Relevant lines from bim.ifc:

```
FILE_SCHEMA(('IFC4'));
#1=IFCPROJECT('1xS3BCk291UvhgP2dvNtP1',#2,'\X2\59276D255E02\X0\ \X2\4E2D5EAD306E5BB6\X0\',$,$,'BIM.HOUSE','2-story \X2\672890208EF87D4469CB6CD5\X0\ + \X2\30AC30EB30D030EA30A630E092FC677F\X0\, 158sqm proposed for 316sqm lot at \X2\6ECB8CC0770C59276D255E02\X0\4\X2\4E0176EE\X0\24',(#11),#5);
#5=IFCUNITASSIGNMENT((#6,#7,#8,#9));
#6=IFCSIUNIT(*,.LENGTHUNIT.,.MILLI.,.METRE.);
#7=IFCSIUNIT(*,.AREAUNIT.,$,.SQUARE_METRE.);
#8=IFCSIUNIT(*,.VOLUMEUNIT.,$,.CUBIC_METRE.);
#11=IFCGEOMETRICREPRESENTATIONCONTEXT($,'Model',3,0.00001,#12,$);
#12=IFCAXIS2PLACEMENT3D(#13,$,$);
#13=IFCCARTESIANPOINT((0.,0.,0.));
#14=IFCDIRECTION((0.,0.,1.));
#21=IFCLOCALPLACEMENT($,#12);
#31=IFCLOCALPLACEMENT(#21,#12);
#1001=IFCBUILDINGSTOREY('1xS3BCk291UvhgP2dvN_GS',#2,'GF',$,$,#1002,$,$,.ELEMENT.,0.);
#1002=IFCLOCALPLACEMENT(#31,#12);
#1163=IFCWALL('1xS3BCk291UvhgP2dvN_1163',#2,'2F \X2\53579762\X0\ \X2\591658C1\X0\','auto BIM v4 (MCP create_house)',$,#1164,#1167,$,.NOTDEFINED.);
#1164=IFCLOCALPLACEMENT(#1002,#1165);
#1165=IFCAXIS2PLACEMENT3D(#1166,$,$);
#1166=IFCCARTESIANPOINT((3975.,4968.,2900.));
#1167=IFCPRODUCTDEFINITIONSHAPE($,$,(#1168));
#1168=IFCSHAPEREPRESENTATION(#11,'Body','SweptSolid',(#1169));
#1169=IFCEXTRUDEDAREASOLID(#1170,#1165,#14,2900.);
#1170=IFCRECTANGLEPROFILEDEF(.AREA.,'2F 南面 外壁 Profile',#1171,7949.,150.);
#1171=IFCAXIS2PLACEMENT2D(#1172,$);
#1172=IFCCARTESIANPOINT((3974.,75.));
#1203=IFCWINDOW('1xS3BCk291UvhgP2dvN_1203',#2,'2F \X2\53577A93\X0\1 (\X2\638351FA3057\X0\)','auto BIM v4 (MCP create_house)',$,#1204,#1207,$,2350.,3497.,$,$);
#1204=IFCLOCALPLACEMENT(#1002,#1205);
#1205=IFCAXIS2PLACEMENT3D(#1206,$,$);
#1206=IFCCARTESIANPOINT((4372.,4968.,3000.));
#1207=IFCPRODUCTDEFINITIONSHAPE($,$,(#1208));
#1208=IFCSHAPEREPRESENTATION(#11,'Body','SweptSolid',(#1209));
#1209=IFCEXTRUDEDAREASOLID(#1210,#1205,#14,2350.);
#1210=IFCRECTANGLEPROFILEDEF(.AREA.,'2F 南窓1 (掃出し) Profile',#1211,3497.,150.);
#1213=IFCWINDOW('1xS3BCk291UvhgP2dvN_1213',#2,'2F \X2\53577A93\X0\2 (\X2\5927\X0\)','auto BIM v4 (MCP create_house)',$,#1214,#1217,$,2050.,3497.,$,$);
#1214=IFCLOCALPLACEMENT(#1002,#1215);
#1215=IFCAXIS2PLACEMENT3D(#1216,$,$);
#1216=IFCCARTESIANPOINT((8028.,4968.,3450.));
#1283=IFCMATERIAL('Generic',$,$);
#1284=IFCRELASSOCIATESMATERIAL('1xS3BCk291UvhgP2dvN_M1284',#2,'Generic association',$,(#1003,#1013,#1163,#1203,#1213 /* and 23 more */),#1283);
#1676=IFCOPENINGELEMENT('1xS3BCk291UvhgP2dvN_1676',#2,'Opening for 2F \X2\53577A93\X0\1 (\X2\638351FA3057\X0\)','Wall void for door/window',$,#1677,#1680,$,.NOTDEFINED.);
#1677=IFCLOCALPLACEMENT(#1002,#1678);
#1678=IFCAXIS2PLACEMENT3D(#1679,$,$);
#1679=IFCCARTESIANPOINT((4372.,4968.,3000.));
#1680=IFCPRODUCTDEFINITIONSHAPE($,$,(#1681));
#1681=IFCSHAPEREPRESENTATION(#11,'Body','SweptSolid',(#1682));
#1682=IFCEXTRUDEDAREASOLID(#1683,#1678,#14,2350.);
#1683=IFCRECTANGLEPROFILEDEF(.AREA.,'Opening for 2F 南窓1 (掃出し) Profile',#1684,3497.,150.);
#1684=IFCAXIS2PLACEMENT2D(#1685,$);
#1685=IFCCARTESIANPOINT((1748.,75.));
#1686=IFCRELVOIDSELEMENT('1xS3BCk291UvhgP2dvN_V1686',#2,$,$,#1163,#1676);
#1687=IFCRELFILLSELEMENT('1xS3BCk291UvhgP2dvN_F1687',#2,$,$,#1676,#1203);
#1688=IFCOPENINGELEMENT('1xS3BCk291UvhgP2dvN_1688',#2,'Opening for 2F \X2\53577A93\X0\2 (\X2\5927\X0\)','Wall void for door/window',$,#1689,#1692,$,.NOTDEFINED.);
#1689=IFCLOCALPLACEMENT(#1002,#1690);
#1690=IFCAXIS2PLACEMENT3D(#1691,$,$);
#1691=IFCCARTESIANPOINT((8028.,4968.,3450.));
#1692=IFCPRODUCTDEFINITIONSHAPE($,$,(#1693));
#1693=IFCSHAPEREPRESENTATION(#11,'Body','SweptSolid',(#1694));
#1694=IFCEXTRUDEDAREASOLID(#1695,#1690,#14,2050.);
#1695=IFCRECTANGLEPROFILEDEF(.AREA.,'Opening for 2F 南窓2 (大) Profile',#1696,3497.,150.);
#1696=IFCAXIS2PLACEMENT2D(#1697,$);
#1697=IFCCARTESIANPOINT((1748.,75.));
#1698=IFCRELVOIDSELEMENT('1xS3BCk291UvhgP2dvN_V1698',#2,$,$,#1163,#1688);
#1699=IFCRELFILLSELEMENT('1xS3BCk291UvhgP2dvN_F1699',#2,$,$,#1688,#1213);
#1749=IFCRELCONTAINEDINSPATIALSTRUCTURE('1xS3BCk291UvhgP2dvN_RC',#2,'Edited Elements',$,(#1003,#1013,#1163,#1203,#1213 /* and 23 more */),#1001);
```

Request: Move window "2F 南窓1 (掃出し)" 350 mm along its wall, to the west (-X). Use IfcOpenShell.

```python
import ifcopenshell
import ifcopenshell.api.geometry
import ifcopenshell.util.placement

model = ifcopenshell.open("bim.ifc")

window = model.by_guid("1xS3BCk291UvhgP2dvN_1203")
opening = window.FillsVoids[0].RelatingOpeningElement
wall = opening.VoidsElements[0].RelatingBuildingElement

wall_matrix = ifcopenshell.util.placement.get_local_placement(wall.ObjectPlacement)
shift = wall_matrix[:3, 0] * -350.0
before = ifcopenshell.util.placement.get_local_placement(window.ObjectPlacement)[:3, 3].copy()

# The window is not placed relative to its opening, so move both.
for product in (opening, window):
    matrix = ifcopenshell.util.placement.get_local_placement(product.ObjectPlacement)
    matrix[:3, 3] += shift
    ifcopenshell.api.geometry.edit_object_placement(model, product=product, matrix=matrix, is_si=False)

after = ifcopenshell.util.placement.get_local_placement(window.ObjectPlacement)[:3, 3]
print("window moved by", (after - before).round(3) + 0.0)

model.write("bim_edited.ifc")
```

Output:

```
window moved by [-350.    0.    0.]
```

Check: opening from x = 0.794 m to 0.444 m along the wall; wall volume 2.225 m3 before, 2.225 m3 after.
